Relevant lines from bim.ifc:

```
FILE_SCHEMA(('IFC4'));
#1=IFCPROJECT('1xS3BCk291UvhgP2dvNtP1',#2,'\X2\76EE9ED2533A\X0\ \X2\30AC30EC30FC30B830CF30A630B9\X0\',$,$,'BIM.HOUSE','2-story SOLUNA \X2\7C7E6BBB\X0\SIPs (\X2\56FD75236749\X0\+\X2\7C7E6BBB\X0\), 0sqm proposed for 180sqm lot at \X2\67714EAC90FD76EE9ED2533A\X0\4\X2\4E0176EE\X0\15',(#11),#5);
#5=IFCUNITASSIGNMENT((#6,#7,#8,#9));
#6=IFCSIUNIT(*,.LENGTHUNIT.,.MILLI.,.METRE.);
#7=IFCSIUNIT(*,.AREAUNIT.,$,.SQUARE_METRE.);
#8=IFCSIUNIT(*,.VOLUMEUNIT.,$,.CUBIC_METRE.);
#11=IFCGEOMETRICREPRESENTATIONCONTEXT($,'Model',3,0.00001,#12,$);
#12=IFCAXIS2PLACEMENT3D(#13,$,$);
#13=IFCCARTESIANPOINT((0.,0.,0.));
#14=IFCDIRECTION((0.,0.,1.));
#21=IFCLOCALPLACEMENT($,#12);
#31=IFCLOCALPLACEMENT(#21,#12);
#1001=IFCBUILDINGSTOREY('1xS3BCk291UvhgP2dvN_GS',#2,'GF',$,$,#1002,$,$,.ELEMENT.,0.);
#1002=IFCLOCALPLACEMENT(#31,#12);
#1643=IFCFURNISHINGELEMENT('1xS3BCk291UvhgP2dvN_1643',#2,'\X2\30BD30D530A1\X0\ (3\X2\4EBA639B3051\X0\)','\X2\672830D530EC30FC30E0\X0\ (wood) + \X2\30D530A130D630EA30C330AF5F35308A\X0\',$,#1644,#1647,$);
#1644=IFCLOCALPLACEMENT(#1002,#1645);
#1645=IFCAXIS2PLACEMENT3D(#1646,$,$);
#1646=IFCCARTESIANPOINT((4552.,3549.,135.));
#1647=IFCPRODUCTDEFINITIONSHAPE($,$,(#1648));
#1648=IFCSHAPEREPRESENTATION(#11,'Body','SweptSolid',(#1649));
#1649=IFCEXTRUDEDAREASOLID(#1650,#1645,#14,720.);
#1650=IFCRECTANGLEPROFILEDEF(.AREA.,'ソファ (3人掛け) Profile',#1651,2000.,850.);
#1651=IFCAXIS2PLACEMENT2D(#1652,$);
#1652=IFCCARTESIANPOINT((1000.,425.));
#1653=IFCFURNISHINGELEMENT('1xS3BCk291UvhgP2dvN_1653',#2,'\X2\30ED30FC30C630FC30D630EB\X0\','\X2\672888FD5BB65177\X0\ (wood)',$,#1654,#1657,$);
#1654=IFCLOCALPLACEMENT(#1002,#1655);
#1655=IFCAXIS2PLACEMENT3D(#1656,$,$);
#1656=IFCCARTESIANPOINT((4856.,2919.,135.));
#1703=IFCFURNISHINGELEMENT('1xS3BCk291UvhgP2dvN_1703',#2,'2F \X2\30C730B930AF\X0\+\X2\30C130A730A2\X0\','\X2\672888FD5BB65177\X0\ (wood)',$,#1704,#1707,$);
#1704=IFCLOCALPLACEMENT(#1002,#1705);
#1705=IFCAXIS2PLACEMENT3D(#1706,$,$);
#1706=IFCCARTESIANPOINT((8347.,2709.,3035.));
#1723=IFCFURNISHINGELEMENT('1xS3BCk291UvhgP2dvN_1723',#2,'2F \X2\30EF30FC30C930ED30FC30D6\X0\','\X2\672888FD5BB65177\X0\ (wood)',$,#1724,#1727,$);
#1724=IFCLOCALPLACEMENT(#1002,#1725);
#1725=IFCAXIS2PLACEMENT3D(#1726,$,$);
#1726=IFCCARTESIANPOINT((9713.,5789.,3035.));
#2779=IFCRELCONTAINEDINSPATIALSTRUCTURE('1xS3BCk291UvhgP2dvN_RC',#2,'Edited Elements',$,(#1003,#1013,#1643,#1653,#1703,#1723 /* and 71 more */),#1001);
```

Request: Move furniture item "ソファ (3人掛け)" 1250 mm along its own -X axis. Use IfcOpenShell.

```python
import ifcopenshell
import ifcopenshell.api.geometry
import ifcopenshell.util.placement
import ifcopenshell.util.unit

model = ifcopenshell.open("bim.ifc")
unit_scale = ifcopenshell.util.unit.calculate_unit_scale(model)

item = model.by_guid("1xS3BCk291UvhgP2dvN_1643")
matrix = ifcopenshell.util.placement.get_local_placement(item.ObjectPlacement)
matrix[:3, 3] -= matrix[:3, 0] * 1.25 / unit_scale
ifcopenshell.api.geometry.edit_object_placement(model, product=item, matrix=matrix, is_si=False)

print(ifcopenshell.util.placement.get_local_placement(item.ObjectPlacement).round(3) + 0.0)

model.write("bim_v2.ifc")
```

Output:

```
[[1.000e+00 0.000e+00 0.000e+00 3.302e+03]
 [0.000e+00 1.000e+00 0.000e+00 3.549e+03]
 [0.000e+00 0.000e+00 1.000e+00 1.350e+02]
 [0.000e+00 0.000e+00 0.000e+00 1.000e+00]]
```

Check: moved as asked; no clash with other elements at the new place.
